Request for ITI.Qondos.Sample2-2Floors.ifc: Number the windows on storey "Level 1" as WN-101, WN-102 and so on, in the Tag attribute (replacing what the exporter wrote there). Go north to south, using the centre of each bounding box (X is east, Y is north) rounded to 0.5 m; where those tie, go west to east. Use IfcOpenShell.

First a look at what the model holds.

```python
import ifcopenshell
import ifcopenshell.util.element
import ifcopenshell.util.placement

model = ifcopenshell.open("ITI.Qondos.Sample2-2Floors.ifc")
print(model.schema)
storey = next(s for s in model.by_type("IfcBuildingStorey") if s.Name == "Level 1")
windows = [e for e in ifcopenshell.util.element.get_decomposition(storey) if e.is_a("IfcWindow")]
for e in sorted(windows, key=lambda e: e.id()):
    origin = ifcopenshell.util.placement.get_local_placement(e.ObjectPlacement)[:3, 3]
    print(e.id(), e.Tag, e.Name, origin.round(2) + 0.0, sep=" | ")
```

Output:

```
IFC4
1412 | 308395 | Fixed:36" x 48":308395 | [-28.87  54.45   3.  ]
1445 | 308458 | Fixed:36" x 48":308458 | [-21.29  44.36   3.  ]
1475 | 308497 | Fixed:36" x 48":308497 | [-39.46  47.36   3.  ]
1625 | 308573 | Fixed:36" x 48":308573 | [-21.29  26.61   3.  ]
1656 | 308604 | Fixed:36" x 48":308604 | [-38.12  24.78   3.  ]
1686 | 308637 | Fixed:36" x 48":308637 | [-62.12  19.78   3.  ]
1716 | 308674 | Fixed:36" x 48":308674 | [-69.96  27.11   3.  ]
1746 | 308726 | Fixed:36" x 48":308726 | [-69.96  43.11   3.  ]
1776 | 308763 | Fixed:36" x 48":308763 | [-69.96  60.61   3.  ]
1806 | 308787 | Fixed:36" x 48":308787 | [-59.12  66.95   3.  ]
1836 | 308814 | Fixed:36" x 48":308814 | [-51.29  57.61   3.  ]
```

```python
import ifcopenshell
import ifcopenshell.geom
import ifcopenshell.util.element
import ifcopenshell.util.shape

model = ifcopenshell.open("ITI.Qondos.Sample2-2Floors.ifc")
settings = ifcopenshell.geom.settings()
settings.set("use-world-coords", True)


def centre(element):
    shape = ifcopenshell.geom.create_shape(settings, element)
    return ifcopenshell.util.shape.get_bbox_centroid(shape.geometry)


storey = next(s for s in model.by_type("IfcBuildingStorey") if s.Name == "Level 1")
windows = [e for e in ifcopenshell.util.element.get_decomposition(storey) if e.is_a("IfcWindow")]

# Insertion points can sit at a corner or the storey origin, so sort by the geometry (in metres).
centres = {e: centre(e) for e in windows}
windows.sort(key=lambda e: (-round(centres[e][1] / 0.5), centres[e][0]))

for i, e in enumerate(windows, start=1):
    number = f"WN-1{i:02d}"
    e.Tag = number
    print(e.id(), number)

model.write("ITI.Qondos.Sample2-2Floors_updated.ifc")
```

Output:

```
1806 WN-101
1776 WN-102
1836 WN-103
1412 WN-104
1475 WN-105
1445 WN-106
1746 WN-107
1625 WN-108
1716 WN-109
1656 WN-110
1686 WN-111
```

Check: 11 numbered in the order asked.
